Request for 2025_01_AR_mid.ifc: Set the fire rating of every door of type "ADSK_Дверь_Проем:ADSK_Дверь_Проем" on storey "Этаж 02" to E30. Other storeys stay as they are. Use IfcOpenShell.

First a look at what the model holds.

```python
import ifcopenshell
import ifcopenshell.util.element

model = ifcopenshell.open("2025_01_AR_mid.ifc")
print(model.schema)
storey = next(s for s in model.by_type("IfcBuildingStorey") if s.Name == "Этаж 02")
doors = [e for e in ifcopenshell.util.element.get_decomposition(storey) if e.is_a("IfcDoor")]
seen = {}
for e in doors:
    element_type = ifcopenshell.util.element.get_type(e)
    key = (element_type.Name if element_type != e and element_type else None, ifcopenshell.util.element.get_pset(e, "Pset_DoorCommon", "FireRating"))
    seen[key] = seen.get(key, 0) + 1
for (name, value), count in sorted(seen.items(), key=str):
    print(count, "x", name, "|", value)
```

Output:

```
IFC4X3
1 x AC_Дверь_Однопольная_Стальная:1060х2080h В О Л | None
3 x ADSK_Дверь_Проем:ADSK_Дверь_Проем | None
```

```python
import ifcopenshell
import ifcopenshell.api.pset
import ifcopenshell.util.element

model = ifcopenshell.open("2025_01_AR_mid.ifc")

storey = next(s for s in model.by_type("IfcBuildingStorey") if s.Name == "Этаж 02")
doors = [e for e in ifcopenshell.util.element.get_decomposition(storey) if e.is_a("IfcDoor")]

count = 0
for e in doors:
    element_type = ifcopenshell.util.element.get_type(e)
    if element_type in (None, e) or element_type.Name != "ADSK_Дверь_Проем:ADSK_Дверь_Проем":
        continue
    # add_pset returns the element's existing set when there is one.
    pset = ifcopenshell.api.pset.add_pset(model, product=e, name="Pset_DoorCommon")
    ifcopenshell.api.pset.edit_pset(model, pset=pset, properties={"FireRating": "E30"})
    count += 1

print(count, "doors updated")

model.write("2025_01_AR_mid_updated.ifc")
```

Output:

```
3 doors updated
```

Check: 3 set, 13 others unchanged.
